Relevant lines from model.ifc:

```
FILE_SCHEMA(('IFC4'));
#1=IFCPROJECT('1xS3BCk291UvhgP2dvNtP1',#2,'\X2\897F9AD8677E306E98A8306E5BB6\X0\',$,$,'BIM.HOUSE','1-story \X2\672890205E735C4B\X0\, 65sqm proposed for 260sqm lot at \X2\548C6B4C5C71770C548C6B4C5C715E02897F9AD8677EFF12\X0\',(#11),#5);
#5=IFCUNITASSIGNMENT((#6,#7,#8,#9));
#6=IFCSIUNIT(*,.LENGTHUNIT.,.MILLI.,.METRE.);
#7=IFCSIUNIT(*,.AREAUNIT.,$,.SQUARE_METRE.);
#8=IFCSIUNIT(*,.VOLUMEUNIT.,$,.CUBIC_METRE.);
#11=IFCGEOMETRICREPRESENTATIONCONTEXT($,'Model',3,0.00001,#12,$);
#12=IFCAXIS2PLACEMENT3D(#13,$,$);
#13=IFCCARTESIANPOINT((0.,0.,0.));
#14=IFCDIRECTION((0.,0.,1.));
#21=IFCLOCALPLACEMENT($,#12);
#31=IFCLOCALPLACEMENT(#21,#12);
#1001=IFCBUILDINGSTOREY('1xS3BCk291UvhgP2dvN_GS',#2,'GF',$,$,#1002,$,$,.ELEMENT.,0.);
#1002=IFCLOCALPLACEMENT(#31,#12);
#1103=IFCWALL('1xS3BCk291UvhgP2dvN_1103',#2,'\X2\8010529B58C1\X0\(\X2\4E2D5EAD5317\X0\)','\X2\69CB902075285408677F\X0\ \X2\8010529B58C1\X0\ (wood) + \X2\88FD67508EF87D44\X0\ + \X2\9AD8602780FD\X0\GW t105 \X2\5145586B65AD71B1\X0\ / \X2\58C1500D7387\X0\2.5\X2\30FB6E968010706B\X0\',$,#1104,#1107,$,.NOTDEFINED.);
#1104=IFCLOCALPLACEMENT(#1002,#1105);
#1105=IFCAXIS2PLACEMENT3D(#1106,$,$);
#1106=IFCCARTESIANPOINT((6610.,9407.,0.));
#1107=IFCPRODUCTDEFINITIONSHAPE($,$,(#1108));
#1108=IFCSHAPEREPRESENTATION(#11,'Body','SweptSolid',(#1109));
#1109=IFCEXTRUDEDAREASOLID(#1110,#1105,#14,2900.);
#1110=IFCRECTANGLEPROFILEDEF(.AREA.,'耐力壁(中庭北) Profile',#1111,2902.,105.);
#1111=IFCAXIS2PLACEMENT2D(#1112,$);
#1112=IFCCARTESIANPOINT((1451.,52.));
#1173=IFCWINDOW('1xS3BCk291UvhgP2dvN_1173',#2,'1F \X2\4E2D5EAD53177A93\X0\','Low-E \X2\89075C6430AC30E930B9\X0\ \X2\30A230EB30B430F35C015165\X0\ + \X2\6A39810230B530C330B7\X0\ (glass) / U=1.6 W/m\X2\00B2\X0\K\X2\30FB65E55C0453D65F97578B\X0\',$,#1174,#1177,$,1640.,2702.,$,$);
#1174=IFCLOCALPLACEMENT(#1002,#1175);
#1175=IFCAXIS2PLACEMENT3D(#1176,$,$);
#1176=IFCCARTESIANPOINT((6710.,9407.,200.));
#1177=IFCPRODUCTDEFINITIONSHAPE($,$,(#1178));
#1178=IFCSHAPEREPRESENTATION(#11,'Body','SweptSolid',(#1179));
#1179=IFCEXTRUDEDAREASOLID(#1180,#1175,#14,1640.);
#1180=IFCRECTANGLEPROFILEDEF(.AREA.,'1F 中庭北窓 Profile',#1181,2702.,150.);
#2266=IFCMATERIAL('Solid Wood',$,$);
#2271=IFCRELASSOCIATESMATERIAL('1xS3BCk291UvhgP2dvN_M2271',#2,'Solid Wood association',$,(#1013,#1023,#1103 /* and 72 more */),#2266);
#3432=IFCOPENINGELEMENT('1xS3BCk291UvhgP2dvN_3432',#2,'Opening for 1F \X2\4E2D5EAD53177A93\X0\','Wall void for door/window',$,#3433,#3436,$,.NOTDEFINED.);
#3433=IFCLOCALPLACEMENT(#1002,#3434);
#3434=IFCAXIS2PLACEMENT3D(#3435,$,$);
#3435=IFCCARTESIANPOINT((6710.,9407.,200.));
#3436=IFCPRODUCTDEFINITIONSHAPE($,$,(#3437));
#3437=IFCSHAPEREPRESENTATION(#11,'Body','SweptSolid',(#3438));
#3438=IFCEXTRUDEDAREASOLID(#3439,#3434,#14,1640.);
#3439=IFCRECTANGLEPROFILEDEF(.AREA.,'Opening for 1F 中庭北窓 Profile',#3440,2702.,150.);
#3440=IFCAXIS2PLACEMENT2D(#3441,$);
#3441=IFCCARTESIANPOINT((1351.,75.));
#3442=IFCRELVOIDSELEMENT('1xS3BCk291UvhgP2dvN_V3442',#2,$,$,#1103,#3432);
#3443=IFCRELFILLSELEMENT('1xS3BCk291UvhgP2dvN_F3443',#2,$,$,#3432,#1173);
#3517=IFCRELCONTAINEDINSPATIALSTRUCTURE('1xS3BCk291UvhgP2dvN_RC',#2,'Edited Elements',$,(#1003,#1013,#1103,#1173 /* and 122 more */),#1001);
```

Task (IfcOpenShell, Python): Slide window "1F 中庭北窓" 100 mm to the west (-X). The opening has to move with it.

```python
import ifcopenshell
import ifcopenshell.api.geometry
import ifcopenshell.util.placement
import ifcopenshell.util.unit

model = ifcopenshell.open("model.ifc")
unit_scale = ifcopenshell.util.unit.calculate_unit_scale(model)

window = model.by_guid("1xS3BCk291UvhgP2dvN_1173")
opening = window.FillsVoids[0].RelatingOpeningElement
wall = opening.VoidsElements[0].RelatingBuildingElement

wall_matrix = ifcopenshell.util.placement.get_local_placement(wall.ObjectPlacement)
shift = wall_matrix[:3, 0] * -0.1 / unit_scale
before = ifcopenshell.util.placement.get_local_placement(window.ObjectPlacement)[:3, 3].copy()

# The window is not placed relative to its opening, so move both.
for product in (opening, window):
    matrix = ifcopenshell.util.placement.get_local_placement(product.ObjectPlacement)
    matrix[:3, 3] += shift
    ifcopenshell.api.geometry.edit_object_placement(model, product=product, matrix=matrix, is_si=False)

after = ifcopenshell.util.placement.get_local_placement(window.ObjectPlacement)[:3, 3]
print("window moved by", (after - before).round(3) + 0.0)

model.write("model_edited.ifc")
```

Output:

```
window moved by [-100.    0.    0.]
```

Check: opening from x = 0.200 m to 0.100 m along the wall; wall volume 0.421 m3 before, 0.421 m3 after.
